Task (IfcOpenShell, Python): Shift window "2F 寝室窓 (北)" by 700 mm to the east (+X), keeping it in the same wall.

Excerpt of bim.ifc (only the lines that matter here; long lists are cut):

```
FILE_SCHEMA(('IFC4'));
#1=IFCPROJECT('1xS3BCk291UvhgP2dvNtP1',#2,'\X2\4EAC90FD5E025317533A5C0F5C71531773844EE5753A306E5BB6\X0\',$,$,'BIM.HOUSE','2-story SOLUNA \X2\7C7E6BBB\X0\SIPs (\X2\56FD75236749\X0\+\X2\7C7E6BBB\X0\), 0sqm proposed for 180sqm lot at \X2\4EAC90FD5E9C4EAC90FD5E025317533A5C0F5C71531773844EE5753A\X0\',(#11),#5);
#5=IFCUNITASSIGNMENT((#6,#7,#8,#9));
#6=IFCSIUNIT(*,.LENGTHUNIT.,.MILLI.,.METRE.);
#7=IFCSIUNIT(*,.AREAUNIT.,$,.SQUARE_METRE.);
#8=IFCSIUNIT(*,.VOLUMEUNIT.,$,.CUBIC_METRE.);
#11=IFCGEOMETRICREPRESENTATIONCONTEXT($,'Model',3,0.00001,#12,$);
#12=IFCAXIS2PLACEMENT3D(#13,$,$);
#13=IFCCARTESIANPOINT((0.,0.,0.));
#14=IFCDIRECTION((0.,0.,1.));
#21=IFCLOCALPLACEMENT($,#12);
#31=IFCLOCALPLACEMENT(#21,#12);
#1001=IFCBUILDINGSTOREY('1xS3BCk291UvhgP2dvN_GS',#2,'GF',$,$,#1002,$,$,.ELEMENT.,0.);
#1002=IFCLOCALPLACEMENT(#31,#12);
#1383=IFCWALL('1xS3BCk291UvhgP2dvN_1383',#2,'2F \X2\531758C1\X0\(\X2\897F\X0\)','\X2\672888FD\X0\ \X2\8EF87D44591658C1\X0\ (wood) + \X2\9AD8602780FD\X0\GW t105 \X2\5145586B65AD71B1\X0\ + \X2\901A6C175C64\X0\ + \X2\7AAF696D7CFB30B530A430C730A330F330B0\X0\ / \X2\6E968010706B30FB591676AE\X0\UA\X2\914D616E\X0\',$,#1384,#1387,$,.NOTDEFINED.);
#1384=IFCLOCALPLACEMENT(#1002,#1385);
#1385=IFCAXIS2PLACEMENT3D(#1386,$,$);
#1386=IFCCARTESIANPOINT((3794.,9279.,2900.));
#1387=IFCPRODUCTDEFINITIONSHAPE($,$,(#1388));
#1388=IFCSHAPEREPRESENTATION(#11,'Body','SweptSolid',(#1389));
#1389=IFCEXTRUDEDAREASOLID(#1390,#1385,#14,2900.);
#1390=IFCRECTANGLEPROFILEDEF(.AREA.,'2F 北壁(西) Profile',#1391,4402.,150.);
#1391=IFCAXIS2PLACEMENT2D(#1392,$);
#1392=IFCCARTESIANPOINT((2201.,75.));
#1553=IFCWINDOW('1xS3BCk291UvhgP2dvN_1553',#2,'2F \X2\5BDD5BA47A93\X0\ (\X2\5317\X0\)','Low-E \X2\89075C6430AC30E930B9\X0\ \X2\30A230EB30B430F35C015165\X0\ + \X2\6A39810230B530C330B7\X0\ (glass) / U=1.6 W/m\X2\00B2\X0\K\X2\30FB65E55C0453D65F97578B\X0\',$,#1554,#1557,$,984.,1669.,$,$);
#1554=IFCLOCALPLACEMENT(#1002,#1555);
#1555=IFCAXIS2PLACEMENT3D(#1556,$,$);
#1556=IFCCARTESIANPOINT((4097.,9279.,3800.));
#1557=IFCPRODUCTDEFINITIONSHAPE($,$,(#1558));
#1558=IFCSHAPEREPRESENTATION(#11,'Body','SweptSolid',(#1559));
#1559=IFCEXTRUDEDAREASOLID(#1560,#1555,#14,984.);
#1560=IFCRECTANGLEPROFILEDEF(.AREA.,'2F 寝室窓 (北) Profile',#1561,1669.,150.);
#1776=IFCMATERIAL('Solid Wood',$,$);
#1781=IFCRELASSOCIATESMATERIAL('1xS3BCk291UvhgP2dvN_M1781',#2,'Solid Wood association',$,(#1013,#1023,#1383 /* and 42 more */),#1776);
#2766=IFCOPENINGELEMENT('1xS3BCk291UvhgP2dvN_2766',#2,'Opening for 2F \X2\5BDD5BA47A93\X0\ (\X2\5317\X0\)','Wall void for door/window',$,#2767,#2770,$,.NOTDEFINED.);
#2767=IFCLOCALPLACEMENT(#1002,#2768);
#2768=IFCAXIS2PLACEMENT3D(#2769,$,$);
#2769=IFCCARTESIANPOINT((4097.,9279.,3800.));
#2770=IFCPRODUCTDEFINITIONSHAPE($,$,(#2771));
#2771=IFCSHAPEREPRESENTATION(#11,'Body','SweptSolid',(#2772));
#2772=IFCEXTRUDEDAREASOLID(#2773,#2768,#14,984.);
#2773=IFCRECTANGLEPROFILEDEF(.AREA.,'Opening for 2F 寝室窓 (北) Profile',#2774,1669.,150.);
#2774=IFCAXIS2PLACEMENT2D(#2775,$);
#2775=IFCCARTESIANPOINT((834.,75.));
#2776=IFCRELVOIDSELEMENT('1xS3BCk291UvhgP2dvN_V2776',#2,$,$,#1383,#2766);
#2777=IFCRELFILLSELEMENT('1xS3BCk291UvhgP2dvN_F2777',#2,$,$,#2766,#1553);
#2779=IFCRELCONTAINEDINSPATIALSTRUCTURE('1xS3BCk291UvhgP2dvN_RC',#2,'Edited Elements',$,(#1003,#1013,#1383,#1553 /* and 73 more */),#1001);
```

```python
import ifcopenshell
import ifcopenshell.api.geometry
import ifcopenshell.util.placement

model = ifcopenshell.open("bim.ifc")

window = model.by_id(1553)
opening = window.FillsVoids[0].RelatingOpeningElement
wall = opening.VoidsElements[0].RelatingBuildingElement

wall_matrix = ifcopenshell.util.placement.get_local_placement(wall.ObjectPlacement)
shift = wall_matrix[:3, 0] * 700.0
before = ifcopenshell.util.placement.get_local_placement(window.ObjectPlacement)[:3, 3].copy()

# The window is not placed relative to its opening, so move both.
for product in (opening, window):
    matrix = ifcopenshell.util.placement.get_local_placement(product.ObjectPlacement)
    matrix[:3, 3] += shift
    ifcopenshell.api.geometry.edit_object_placement(model, product=product, matrix=matrix, is_si=False)

after = ifcopenshell.util.placement.get_local_placement(window.ObjectPlacement)[:3, 3]
print("window moved by", (after - before).round(3) + 0.0)

model.write("bim_updated.ifc")
```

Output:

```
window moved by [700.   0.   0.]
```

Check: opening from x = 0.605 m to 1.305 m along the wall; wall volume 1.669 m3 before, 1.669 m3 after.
